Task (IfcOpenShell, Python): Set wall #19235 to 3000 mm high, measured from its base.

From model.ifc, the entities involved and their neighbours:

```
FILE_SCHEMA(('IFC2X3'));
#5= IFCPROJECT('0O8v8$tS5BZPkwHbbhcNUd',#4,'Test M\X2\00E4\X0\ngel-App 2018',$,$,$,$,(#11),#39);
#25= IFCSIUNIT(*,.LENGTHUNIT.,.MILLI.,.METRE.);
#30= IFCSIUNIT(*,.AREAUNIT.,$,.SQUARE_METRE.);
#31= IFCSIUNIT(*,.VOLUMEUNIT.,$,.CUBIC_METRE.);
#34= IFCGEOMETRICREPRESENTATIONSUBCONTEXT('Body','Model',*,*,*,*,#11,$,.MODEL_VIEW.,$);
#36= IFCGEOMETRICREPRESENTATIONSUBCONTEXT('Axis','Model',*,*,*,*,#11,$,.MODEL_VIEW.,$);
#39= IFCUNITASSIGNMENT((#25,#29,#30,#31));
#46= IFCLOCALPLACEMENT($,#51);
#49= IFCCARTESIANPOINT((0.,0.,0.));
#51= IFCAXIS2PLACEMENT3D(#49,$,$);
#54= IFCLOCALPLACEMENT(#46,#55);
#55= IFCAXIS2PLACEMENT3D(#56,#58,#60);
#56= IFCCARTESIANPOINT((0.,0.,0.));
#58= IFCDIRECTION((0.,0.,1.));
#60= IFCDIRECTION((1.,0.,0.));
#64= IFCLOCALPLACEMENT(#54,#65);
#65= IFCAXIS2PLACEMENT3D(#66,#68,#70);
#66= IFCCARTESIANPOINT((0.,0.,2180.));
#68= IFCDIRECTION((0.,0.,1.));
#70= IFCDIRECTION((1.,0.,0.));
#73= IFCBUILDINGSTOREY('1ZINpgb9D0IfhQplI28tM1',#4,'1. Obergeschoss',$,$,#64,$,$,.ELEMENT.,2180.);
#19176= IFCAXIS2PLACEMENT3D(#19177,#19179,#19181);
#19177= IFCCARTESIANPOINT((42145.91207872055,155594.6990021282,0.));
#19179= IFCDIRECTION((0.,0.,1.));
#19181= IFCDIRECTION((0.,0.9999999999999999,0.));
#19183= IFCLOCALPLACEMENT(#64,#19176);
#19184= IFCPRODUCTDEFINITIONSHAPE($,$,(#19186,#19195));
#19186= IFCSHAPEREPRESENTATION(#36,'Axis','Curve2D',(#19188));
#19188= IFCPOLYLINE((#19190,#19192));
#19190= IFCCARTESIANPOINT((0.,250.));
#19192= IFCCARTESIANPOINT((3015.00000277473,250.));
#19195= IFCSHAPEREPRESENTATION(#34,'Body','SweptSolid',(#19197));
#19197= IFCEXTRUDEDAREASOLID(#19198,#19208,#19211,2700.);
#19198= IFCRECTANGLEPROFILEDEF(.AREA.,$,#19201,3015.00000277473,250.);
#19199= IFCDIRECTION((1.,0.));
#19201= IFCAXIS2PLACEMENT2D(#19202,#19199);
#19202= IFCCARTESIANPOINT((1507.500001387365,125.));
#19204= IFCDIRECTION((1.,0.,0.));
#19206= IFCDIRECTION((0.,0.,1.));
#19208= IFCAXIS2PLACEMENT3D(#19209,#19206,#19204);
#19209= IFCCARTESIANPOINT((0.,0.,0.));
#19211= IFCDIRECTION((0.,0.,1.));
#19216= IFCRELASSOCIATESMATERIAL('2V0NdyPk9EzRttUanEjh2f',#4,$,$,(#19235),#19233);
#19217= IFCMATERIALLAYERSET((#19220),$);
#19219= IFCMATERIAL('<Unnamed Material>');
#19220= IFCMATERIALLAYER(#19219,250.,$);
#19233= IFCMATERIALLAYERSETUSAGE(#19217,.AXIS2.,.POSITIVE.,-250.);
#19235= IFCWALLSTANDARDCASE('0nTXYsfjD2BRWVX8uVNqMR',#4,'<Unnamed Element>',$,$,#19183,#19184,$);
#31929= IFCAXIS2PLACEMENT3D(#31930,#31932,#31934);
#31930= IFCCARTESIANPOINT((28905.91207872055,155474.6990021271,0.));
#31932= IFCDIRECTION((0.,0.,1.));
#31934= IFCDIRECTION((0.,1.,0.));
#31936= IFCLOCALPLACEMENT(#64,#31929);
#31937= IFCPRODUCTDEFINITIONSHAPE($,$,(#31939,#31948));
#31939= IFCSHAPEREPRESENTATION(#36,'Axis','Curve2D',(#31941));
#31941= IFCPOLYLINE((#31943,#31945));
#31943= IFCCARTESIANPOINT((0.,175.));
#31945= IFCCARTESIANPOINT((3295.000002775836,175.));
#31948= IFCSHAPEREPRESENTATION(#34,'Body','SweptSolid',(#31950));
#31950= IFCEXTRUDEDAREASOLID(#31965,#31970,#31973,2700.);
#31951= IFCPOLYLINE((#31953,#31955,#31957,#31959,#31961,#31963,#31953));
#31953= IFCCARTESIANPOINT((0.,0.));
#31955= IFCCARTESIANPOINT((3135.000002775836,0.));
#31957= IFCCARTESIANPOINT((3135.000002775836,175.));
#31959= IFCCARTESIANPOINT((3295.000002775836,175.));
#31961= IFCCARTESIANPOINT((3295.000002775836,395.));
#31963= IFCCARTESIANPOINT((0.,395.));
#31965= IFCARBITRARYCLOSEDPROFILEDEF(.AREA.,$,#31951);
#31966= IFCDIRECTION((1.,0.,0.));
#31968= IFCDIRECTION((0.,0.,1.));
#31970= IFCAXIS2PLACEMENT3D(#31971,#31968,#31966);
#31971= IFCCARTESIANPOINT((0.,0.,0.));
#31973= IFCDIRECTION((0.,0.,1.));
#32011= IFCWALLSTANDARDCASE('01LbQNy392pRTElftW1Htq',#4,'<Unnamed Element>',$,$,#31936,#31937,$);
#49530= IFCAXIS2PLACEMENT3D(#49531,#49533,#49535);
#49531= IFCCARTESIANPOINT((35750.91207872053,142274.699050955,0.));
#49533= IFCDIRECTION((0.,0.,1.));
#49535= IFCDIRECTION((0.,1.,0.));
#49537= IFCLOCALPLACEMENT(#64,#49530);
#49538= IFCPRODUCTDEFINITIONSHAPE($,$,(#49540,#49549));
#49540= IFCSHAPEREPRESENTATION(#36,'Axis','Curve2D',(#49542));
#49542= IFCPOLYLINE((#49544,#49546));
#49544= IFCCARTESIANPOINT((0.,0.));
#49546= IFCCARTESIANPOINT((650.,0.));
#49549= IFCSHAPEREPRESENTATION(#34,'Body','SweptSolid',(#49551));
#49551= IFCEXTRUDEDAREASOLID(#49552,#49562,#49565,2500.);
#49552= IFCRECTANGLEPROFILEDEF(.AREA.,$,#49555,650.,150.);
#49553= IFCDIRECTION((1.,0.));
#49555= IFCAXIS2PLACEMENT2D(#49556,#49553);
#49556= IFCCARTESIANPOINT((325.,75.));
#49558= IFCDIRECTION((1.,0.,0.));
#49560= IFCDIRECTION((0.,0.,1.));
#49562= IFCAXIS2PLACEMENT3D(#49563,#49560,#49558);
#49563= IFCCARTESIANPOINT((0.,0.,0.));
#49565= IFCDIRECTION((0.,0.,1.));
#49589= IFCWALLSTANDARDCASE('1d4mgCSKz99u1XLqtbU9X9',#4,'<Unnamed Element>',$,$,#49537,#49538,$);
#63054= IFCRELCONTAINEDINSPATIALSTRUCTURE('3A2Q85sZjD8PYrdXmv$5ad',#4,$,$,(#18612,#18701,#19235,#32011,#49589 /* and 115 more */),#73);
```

```python
import ifcopenshell
import ifcopenshell.geom
import ifcopenshell.util.representation
import ifcopenshell.util.shape

model = ifcopenshell.open("model.ifc")
settings = ifcopenshell.geom.settings()


def volume(element):
    """Net volume in cubic metres, openings subtracted."""
    shape = ifcopenshell.geom.create_shape(settings, element)
    return ifcopenshell.util.shape.get_volume(shape.geometry)


wall = model.by_id(19235)
before = volume(wall)

body = ifcopenshell.util.representation.get_representation(wall, "Model", "Body")
solid = body.Items[0]
old_height = solid.Depth
solid.Depth = 3000.0
after = volume(wall)

print(f"height {old_height:g} -> {solid.Depth:g}, volume {before:.3f} -> {after:.3f} m3")

model.write("model_edited.ifc")
```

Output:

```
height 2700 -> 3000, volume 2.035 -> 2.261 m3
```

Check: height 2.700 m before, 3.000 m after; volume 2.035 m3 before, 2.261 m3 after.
